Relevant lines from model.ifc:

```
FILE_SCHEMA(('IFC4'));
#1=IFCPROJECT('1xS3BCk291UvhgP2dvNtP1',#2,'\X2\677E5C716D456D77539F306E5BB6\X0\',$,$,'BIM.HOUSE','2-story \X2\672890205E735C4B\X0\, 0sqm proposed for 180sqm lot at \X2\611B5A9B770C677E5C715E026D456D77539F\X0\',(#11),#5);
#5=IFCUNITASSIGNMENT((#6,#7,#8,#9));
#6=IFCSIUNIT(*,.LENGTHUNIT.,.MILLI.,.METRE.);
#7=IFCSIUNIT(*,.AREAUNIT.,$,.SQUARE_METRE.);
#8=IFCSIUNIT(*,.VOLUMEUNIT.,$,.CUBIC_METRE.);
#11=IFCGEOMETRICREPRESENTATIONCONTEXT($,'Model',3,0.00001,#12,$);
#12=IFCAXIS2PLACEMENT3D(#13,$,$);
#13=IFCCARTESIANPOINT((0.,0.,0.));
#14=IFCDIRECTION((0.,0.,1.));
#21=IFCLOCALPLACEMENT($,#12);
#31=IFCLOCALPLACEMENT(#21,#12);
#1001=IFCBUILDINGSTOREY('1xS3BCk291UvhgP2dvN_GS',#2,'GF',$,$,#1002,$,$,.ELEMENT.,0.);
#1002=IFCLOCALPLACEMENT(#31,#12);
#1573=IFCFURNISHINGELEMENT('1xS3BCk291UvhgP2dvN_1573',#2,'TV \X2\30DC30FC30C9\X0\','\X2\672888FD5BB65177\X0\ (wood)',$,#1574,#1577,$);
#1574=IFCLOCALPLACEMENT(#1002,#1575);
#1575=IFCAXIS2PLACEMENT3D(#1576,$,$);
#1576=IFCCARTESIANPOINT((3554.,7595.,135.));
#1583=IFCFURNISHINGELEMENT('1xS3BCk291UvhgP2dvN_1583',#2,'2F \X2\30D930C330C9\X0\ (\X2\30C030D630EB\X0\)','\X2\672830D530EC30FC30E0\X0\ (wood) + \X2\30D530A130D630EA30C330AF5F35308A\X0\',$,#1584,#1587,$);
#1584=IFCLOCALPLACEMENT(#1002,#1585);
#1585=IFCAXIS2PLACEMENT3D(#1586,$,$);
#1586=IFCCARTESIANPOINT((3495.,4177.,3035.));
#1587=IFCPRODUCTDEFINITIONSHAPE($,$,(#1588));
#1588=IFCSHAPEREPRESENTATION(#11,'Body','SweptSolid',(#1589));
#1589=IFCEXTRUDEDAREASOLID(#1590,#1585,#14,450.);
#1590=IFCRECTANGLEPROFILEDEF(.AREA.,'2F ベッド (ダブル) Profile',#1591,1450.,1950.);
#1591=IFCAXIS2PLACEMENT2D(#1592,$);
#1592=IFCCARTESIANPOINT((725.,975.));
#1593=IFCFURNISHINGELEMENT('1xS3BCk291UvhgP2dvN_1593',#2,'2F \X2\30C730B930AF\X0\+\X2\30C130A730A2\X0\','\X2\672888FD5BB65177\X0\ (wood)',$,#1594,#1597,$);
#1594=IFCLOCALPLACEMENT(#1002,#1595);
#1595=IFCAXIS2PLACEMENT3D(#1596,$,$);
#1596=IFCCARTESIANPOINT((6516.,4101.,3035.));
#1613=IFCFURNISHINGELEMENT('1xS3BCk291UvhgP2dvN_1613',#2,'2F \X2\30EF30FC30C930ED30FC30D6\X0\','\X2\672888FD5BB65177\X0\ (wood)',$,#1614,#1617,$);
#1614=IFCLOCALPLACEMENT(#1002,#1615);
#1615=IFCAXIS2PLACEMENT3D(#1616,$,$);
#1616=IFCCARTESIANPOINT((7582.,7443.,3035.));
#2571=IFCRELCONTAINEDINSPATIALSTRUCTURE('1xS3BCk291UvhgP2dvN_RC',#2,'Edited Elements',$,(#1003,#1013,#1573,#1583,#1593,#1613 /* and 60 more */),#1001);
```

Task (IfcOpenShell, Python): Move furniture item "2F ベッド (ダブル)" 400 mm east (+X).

```python
import ifcopenshell
import ifcopenshell.api.geometry
import ifcopenshell.util.placement
import ifcopenshell.util.unit

model = ifcopenshell.open("model.ifc")
unit_scale = ifcopenshell.util.unit.calculate_unit_scale(model)

item = model.by_guid("1xS3BCk291UvhgP2dvN_1583")
matrix = ifcopenshell.util.placement.get_local_placement(item.ObjectPlacement)
matrix[0, 3] += 0.4 / unit_scale
ifcopenshell.api.geometry.edit_object_placement(model, product=item, matrix=matrix, is_si=False)

print(ifcopenshell.util.placement.get_local_placement(item.ObjectPlacement).round(3) + 0.0)

model.write("model_updated.ifc")
```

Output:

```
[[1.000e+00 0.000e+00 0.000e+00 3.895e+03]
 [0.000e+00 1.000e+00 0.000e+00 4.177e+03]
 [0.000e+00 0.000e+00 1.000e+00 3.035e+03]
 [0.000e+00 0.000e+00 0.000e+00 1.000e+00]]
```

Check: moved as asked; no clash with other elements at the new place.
